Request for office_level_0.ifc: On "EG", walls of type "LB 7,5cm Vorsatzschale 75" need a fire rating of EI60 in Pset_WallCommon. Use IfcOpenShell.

First a look at what the model holds.

```python
import ifcopenshell
import ifcopenshell.util.element

model = ifcopenshell.open("office_level_0.ifc")
print(model.schema)
storey = next(s for s in model.by_type("IfcBuildingStorey") if s.Name == "EG")
walls = [e for e in ifcopenshell.util.element.get_decomposition(storey) if e.is_a("IfcWall")]
seen = {}
for e in walls:
    element_type = ifcopenshell.util.element.get_type(e)
    key = (element_type.Name if element_type != e and element_type else None, ifcopenshell.util.element.get_pset(e, "Pset_WallCommon", "FireRating"))
    seen[key] = seen.get(key, 0) + 1
for (name, value), count in sorted(seen.items(), key=str):
    print(count, "x", name, "|", value)
```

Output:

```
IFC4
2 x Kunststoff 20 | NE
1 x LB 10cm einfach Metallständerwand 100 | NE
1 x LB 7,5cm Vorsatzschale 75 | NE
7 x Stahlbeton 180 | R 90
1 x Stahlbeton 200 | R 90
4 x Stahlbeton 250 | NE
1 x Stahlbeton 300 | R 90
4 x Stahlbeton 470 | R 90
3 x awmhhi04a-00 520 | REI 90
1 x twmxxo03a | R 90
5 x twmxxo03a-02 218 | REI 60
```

```python
import ifcopenshell
import ifcopenshell.api.pset
import ifcopenshell.util.element

model = ifcopenshell.open("office_level_0.ifc")

storey = next(s for s in model.by_type("IfcBuildingStorey") if s.Name == "EG")
walls = [e for e in ifcopenshell.util.element.get_decomposition(storey) if e.is_a("IfcWall")]

count = 0
for e in walls:
    element_type = ifcopenshell.util.element.get_type(e)
    if element_type in (None, e) or element_type.Name != "LB 7,5cm Vorsatzschale 75":
        continue
    # add_pset returns the element's existing set when there is one.
    pset = ifcopenshell.api.pset.add_pset(model, product=e, name="Pset_WallCommon")
    ifcopenshell.api.pset.edit_pset(model, pset=pset, properties={"FireRating": "EI60"})
    count += 1

print(count, "walls updated")

model.write("office_level_0_rev.ifc")
```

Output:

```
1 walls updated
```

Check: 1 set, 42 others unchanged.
